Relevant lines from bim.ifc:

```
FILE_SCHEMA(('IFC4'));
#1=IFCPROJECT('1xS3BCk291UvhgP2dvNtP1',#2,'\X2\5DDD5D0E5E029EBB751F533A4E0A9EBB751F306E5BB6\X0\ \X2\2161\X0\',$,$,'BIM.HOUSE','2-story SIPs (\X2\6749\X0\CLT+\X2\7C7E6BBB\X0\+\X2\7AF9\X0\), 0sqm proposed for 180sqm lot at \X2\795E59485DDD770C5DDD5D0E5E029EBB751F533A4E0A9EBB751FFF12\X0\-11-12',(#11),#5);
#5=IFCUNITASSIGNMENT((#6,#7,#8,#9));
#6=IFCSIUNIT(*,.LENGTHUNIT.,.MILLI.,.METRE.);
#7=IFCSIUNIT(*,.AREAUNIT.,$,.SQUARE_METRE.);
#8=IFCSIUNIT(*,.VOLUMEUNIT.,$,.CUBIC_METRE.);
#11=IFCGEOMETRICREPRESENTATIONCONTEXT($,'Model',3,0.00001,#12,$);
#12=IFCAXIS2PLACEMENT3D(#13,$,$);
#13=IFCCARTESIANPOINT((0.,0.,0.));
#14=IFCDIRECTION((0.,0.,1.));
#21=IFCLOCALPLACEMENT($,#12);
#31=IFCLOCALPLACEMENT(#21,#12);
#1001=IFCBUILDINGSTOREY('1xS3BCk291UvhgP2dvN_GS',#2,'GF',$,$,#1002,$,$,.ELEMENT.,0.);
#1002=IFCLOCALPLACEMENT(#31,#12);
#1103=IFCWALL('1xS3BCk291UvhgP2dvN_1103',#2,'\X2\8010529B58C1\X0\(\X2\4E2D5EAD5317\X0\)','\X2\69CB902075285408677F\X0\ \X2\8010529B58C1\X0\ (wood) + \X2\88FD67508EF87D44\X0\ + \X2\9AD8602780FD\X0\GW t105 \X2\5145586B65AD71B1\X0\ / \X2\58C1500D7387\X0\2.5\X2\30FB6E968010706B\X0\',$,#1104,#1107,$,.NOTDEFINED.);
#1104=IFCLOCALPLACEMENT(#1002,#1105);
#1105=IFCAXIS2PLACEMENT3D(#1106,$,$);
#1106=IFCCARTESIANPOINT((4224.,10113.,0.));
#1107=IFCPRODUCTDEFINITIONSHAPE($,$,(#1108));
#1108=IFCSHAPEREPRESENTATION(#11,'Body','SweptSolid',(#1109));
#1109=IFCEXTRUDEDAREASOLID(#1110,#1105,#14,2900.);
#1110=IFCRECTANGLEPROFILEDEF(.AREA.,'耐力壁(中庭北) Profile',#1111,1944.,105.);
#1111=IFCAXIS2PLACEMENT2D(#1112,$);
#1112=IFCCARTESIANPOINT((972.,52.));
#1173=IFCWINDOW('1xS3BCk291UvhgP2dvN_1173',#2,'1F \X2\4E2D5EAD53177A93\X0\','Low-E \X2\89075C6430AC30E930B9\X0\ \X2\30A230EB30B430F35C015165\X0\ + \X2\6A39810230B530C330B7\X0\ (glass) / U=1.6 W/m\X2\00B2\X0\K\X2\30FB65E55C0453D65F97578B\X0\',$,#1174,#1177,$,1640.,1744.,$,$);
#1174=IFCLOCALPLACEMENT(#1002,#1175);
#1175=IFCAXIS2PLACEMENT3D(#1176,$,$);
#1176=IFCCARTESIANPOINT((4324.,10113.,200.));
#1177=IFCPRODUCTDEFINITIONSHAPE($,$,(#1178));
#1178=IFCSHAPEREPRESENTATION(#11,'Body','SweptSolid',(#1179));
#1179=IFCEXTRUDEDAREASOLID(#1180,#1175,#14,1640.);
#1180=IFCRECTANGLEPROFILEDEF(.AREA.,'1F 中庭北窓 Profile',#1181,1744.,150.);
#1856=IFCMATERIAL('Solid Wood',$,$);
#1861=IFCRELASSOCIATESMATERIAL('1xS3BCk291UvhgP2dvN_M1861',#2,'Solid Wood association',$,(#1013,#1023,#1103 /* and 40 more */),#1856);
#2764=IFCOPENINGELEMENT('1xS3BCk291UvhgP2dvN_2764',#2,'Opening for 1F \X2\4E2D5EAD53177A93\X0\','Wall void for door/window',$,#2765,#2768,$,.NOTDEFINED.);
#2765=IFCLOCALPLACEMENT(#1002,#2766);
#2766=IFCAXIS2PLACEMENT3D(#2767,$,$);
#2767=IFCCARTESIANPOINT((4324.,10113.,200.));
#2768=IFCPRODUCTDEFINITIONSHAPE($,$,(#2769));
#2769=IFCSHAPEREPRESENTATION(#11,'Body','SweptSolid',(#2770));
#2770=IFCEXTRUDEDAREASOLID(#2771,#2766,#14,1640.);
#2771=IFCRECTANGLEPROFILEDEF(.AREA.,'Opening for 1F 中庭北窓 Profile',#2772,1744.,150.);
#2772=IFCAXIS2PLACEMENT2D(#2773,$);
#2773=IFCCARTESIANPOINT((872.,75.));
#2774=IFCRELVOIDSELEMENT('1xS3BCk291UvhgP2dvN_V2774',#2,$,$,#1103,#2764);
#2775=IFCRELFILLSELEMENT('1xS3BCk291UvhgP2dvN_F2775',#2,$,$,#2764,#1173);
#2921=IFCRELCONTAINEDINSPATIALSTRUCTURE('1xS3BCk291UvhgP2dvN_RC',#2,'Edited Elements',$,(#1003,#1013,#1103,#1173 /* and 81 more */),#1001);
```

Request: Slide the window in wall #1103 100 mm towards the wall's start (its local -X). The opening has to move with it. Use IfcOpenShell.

```python
import ifcopenshell
import ifcopenshell.api.geometry
import ifcopenshell.util.placement

model = ifcopenshell.open("bim.ifc")

window = model.by_guid("1xS3BCk291UvhgP2dvN_1173")
opening = window.FillsVoids[0].RelatingOpeningElement
wall = opening.VoidsElements[0].RelatingBuildingElement

wall_matrix = ifcopenshell.util.placement.get_local_placement(wall.ObjectPlacement)
shift = wall_matrix[:3, 0] * -100.0
before = ifcopenshell.util.placement.get_local_placement(window.ObjectPlacement)[:3, 3].copy()

# The window is not placed relative to its opening, so move both.
for product in (opening, window):
    matrix = ifcopenshell.util.placement.get_local_placement(product.ObjectPlacement)
    matrix[:3, 3] += shift
    ifcopenshell.api.geometry.edit_object_placement(model, product=product, matrix=matrix, is_si=False)

after = ifcopenshell.util.placement.get_local_placement(window.ObjectPlacement)[:3, 3]
print("window moved by", (after - before).round(3) + 0.0)

model.write("bim_v2.ifc")
```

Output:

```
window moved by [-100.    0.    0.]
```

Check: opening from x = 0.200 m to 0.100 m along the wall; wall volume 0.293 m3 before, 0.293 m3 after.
